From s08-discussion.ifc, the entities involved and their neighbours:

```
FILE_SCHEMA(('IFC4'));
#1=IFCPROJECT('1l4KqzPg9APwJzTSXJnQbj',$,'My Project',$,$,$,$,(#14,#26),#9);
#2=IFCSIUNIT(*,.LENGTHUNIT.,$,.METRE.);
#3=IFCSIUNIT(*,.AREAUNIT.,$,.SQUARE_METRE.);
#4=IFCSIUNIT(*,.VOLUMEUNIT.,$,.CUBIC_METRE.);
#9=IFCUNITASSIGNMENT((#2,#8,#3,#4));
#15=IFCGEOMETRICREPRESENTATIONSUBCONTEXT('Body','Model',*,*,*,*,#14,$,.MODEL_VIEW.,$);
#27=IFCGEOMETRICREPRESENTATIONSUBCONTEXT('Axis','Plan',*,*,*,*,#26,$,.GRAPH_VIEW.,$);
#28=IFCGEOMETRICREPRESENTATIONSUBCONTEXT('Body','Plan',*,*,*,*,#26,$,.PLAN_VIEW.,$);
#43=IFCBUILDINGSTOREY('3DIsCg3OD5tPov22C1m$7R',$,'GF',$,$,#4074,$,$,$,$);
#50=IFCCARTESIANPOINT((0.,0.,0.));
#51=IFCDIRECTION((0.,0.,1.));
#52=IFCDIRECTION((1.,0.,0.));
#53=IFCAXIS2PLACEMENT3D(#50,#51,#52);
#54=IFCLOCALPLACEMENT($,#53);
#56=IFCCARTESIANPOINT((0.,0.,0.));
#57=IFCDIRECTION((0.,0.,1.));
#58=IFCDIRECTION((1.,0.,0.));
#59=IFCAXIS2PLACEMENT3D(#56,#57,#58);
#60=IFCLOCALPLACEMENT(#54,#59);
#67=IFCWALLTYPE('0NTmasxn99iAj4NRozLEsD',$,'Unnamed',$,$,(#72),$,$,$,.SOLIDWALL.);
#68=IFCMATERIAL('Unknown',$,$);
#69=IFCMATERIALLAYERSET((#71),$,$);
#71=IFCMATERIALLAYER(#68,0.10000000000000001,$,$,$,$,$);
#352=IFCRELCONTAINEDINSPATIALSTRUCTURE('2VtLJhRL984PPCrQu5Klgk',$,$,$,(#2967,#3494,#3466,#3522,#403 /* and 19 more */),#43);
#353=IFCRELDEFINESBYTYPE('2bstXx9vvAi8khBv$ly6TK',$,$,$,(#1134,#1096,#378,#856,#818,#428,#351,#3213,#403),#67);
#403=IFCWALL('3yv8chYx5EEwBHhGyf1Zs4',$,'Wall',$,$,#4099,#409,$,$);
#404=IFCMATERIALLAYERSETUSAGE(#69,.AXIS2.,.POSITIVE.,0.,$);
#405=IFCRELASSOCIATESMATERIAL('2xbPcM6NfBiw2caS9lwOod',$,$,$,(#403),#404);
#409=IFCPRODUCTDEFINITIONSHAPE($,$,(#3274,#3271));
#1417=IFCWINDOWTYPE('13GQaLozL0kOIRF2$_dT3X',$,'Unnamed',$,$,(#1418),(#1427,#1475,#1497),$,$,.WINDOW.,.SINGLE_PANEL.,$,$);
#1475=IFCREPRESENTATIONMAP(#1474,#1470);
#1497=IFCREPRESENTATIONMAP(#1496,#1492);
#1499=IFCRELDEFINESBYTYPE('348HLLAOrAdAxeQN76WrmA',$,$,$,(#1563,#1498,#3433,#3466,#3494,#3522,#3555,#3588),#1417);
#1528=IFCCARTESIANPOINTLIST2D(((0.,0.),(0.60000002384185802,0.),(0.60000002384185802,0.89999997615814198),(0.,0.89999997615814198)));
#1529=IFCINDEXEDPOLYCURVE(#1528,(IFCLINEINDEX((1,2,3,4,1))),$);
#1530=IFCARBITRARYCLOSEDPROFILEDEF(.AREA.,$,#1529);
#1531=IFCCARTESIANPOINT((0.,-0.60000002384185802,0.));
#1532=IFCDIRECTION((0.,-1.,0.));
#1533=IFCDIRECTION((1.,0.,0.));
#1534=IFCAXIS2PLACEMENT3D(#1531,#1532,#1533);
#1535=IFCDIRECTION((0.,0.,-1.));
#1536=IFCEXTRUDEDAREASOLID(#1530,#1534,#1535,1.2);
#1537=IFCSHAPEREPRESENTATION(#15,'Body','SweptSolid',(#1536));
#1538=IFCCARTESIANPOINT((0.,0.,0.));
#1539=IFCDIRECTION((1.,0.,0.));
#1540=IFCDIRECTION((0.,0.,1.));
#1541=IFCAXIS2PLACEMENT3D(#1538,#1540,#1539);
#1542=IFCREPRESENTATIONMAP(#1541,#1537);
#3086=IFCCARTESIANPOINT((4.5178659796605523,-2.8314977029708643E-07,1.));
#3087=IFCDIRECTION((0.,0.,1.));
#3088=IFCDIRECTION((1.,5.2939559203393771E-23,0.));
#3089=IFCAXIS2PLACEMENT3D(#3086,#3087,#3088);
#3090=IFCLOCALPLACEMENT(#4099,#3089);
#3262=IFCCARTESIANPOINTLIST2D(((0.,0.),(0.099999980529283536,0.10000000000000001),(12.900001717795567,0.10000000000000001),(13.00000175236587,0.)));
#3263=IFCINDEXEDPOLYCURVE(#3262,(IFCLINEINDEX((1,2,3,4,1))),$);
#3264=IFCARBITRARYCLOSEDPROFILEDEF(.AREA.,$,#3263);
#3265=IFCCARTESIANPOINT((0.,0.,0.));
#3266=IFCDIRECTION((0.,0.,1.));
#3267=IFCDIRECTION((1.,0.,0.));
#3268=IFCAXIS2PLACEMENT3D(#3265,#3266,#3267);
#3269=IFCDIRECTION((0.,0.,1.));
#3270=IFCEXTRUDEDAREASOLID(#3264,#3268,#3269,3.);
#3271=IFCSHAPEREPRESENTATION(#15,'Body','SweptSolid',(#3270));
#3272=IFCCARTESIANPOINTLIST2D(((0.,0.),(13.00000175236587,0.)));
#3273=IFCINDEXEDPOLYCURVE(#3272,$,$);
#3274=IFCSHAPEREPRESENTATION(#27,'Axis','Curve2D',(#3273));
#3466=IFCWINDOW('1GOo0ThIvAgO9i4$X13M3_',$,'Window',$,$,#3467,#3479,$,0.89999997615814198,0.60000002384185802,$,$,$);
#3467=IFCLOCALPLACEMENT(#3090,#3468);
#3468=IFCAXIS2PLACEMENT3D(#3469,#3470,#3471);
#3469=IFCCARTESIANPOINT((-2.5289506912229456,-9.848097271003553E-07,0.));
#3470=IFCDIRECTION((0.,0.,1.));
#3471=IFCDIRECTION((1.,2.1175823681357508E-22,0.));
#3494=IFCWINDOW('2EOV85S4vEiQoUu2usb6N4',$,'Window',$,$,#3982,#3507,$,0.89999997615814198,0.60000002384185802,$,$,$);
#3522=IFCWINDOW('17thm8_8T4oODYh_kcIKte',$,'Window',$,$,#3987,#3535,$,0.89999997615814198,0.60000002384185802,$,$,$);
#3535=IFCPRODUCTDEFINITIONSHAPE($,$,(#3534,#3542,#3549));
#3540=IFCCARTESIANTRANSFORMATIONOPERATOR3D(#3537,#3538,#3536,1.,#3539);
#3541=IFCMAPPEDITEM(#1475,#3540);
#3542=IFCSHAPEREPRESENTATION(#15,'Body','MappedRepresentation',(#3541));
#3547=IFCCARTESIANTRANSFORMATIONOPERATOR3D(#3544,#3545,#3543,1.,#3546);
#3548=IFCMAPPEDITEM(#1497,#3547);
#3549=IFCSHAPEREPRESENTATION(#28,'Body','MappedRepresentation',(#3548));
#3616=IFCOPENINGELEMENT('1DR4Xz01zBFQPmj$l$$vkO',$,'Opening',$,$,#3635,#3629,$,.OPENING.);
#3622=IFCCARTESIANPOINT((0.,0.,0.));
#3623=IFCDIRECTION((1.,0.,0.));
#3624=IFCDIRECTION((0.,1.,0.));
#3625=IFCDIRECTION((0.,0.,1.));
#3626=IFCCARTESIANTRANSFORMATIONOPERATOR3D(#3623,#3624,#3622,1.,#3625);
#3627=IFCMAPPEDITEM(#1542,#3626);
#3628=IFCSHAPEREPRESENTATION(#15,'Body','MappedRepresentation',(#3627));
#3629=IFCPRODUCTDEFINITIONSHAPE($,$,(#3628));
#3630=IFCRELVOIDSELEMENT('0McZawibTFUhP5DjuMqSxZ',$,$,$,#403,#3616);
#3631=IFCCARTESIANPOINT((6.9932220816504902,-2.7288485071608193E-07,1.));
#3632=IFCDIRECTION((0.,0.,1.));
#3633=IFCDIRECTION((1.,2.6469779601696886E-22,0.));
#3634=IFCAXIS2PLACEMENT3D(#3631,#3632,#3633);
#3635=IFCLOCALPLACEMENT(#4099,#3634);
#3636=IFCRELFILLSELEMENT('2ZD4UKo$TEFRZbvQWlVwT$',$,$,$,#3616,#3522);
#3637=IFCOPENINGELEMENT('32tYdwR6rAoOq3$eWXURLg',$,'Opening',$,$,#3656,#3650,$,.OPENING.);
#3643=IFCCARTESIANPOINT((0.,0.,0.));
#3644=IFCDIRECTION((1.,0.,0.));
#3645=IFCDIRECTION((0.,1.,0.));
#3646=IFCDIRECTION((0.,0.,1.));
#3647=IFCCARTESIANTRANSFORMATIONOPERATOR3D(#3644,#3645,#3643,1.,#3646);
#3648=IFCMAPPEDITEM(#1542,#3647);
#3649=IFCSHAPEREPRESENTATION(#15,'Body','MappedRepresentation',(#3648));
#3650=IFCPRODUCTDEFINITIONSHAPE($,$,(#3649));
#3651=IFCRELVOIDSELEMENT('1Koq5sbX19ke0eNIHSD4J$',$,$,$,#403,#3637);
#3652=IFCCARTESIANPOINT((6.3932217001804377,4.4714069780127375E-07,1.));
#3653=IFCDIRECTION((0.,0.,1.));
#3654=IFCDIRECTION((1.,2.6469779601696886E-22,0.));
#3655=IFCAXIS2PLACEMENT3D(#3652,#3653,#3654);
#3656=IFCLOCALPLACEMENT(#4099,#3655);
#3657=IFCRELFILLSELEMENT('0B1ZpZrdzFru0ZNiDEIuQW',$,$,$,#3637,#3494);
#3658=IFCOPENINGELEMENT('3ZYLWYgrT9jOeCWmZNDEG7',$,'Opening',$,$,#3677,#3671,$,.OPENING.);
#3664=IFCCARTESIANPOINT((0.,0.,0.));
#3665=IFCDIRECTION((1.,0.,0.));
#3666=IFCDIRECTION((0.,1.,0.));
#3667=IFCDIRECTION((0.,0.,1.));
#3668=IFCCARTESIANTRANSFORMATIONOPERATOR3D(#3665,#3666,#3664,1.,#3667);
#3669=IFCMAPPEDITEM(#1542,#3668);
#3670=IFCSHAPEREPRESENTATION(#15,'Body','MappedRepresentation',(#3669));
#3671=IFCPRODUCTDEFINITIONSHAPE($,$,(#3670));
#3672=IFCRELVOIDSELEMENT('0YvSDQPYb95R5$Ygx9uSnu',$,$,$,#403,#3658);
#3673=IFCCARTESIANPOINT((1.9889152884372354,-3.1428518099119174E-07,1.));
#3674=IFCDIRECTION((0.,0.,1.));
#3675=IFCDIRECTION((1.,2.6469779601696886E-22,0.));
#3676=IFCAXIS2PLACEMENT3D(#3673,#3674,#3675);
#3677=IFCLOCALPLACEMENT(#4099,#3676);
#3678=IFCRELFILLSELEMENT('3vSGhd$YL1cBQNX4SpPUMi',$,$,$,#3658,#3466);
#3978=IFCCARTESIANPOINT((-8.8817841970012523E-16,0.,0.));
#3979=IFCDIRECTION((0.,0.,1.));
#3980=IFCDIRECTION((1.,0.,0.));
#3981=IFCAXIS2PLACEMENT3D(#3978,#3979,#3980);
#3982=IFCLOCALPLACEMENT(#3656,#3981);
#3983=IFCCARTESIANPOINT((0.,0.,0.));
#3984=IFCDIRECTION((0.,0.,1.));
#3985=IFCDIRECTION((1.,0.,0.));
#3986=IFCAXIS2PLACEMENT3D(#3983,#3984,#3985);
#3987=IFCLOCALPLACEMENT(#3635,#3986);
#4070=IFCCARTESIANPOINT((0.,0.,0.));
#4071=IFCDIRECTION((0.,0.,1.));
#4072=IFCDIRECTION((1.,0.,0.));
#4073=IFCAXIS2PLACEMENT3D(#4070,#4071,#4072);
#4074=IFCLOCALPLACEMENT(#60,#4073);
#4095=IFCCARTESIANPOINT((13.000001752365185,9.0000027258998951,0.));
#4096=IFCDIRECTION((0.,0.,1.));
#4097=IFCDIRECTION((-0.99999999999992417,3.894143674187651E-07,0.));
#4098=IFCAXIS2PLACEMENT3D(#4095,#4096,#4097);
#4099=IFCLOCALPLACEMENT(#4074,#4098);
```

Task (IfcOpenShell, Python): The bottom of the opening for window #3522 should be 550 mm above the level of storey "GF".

```python
import numpy as np
import ifcopenshell
import ifcopenshell.api.geometry
import ifcopenshell.geom
import ifcopenshell.util.element
import ifcopenshell.util.placement
import ifcopenshell.util.shape
import ifcopenshell.util.unit

model = ifcopenshell.open("s08-discussion.ifc")
unit_scale = ifcopenshell.util.unit.calculate_unit_scale(model)

window = model.by_id(3522)
opening = window.FillsVoids[0].RelatingOpeningElement
storey = ifcopenshell.util.element.get_container(window, ifc_class="IfcBuildingStorey")
level = ifcopenshell.util.placement.get_local_placement(storey.ObjectPlacement)[2, 3]

# The opening's origin need not be at the sill, so measure its lowest point.
shape = ifcopenshell.geom.create_shape(ifcopenshell.geom.settings(), opening)
bottom = ifcopenshell.util.shape.get_shape_bottom_elevation(shape, shape.geometry) / unit_scale
dz = level + 0.55 - bottom

shift = np.array([0.0, 0.0, dz])
# The window is placed relative to its opening, so it follows when the opening moves.
matrix = ifcopenshell.util.placement.get_local_placement(opening.ObjectPlacement)
matrix[:3, 3] += shift
ifcopenshell.api.geometry.edit_object_placement(
    model, product=opening, matrix=matrix, is_si=False, should_transform_children=True
)

print(f"moved by {dz * unit_scale:+.3f} m")

model.write("s08-discussion_rev.ifc")
```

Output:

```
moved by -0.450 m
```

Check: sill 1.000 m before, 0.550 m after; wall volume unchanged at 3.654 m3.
